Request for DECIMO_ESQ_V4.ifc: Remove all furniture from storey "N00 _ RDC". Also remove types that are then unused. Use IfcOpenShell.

First a look at what the model holds.

```python
import ifcopenshell
import ifcopenshell.util.element

model = ifcopenshell.open("DECIMO_ESQ_V4.ifc")
print(model.schema)
storey = next(s for s in model.by_type("IfcBuildingStorey") if s.Name == "N00 _ RDC")
furniture = [e for e in ifcopenshell.util.element.get_decomposition(storey) if e.is_a("IfcFurnishingElement")]
seen = {}
for e in furniture:
    element_type = ifcopenshell.util.element.get_type(e)
    name = element_type.Name if element_type not in (None, e) else None
    seen[name] = seen.get(name, 0) + 1
for name, count in sorted(seen.items(), key=str):
    print(count, "x", name)
```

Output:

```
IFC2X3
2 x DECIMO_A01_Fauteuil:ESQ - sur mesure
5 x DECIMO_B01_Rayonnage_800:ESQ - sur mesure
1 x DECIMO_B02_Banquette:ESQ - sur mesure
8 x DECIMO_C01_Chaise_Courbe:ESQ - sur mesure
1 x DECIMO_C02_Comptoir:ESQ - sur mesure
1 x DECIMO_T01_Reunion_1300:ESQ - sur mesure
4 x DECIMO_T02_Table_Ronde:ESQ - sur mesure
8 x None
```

```python
import ifcopenshell
import ifcopenshell.api.root
import ifcopenshell.util.element

model = ifcopenshell.open("DECIMO_ESQ_V4.ifc")

storey = next(s for s in model.by_type("IfcBuildingStorey") if s.Name == "N00 _ RDC")
furniture = [e for e in ifcopenshell.util.element.get_decomposition(storey) if e.is_a("IfcFurnishingElement")]
types = {ifcopenshell.util.element.get_type(e) for e in furniture} - {None, *furniture}

for e in furniture:
    ifcopenshell.api.root.remove_product(model, product=e)
print(len(furniture), "removed")

unused = [t for t in types if not ifcopenshell.util.element.get_types(t)]
for t in unused:
    ifcopenshell.api.root.remove_product(model, product=t)
print(len(unused), "unused types removed")

model.write("DECIMO_ESQ_V4_updated.ifc")
```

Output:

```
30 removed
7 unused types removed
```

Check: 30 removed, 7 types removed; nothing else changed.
